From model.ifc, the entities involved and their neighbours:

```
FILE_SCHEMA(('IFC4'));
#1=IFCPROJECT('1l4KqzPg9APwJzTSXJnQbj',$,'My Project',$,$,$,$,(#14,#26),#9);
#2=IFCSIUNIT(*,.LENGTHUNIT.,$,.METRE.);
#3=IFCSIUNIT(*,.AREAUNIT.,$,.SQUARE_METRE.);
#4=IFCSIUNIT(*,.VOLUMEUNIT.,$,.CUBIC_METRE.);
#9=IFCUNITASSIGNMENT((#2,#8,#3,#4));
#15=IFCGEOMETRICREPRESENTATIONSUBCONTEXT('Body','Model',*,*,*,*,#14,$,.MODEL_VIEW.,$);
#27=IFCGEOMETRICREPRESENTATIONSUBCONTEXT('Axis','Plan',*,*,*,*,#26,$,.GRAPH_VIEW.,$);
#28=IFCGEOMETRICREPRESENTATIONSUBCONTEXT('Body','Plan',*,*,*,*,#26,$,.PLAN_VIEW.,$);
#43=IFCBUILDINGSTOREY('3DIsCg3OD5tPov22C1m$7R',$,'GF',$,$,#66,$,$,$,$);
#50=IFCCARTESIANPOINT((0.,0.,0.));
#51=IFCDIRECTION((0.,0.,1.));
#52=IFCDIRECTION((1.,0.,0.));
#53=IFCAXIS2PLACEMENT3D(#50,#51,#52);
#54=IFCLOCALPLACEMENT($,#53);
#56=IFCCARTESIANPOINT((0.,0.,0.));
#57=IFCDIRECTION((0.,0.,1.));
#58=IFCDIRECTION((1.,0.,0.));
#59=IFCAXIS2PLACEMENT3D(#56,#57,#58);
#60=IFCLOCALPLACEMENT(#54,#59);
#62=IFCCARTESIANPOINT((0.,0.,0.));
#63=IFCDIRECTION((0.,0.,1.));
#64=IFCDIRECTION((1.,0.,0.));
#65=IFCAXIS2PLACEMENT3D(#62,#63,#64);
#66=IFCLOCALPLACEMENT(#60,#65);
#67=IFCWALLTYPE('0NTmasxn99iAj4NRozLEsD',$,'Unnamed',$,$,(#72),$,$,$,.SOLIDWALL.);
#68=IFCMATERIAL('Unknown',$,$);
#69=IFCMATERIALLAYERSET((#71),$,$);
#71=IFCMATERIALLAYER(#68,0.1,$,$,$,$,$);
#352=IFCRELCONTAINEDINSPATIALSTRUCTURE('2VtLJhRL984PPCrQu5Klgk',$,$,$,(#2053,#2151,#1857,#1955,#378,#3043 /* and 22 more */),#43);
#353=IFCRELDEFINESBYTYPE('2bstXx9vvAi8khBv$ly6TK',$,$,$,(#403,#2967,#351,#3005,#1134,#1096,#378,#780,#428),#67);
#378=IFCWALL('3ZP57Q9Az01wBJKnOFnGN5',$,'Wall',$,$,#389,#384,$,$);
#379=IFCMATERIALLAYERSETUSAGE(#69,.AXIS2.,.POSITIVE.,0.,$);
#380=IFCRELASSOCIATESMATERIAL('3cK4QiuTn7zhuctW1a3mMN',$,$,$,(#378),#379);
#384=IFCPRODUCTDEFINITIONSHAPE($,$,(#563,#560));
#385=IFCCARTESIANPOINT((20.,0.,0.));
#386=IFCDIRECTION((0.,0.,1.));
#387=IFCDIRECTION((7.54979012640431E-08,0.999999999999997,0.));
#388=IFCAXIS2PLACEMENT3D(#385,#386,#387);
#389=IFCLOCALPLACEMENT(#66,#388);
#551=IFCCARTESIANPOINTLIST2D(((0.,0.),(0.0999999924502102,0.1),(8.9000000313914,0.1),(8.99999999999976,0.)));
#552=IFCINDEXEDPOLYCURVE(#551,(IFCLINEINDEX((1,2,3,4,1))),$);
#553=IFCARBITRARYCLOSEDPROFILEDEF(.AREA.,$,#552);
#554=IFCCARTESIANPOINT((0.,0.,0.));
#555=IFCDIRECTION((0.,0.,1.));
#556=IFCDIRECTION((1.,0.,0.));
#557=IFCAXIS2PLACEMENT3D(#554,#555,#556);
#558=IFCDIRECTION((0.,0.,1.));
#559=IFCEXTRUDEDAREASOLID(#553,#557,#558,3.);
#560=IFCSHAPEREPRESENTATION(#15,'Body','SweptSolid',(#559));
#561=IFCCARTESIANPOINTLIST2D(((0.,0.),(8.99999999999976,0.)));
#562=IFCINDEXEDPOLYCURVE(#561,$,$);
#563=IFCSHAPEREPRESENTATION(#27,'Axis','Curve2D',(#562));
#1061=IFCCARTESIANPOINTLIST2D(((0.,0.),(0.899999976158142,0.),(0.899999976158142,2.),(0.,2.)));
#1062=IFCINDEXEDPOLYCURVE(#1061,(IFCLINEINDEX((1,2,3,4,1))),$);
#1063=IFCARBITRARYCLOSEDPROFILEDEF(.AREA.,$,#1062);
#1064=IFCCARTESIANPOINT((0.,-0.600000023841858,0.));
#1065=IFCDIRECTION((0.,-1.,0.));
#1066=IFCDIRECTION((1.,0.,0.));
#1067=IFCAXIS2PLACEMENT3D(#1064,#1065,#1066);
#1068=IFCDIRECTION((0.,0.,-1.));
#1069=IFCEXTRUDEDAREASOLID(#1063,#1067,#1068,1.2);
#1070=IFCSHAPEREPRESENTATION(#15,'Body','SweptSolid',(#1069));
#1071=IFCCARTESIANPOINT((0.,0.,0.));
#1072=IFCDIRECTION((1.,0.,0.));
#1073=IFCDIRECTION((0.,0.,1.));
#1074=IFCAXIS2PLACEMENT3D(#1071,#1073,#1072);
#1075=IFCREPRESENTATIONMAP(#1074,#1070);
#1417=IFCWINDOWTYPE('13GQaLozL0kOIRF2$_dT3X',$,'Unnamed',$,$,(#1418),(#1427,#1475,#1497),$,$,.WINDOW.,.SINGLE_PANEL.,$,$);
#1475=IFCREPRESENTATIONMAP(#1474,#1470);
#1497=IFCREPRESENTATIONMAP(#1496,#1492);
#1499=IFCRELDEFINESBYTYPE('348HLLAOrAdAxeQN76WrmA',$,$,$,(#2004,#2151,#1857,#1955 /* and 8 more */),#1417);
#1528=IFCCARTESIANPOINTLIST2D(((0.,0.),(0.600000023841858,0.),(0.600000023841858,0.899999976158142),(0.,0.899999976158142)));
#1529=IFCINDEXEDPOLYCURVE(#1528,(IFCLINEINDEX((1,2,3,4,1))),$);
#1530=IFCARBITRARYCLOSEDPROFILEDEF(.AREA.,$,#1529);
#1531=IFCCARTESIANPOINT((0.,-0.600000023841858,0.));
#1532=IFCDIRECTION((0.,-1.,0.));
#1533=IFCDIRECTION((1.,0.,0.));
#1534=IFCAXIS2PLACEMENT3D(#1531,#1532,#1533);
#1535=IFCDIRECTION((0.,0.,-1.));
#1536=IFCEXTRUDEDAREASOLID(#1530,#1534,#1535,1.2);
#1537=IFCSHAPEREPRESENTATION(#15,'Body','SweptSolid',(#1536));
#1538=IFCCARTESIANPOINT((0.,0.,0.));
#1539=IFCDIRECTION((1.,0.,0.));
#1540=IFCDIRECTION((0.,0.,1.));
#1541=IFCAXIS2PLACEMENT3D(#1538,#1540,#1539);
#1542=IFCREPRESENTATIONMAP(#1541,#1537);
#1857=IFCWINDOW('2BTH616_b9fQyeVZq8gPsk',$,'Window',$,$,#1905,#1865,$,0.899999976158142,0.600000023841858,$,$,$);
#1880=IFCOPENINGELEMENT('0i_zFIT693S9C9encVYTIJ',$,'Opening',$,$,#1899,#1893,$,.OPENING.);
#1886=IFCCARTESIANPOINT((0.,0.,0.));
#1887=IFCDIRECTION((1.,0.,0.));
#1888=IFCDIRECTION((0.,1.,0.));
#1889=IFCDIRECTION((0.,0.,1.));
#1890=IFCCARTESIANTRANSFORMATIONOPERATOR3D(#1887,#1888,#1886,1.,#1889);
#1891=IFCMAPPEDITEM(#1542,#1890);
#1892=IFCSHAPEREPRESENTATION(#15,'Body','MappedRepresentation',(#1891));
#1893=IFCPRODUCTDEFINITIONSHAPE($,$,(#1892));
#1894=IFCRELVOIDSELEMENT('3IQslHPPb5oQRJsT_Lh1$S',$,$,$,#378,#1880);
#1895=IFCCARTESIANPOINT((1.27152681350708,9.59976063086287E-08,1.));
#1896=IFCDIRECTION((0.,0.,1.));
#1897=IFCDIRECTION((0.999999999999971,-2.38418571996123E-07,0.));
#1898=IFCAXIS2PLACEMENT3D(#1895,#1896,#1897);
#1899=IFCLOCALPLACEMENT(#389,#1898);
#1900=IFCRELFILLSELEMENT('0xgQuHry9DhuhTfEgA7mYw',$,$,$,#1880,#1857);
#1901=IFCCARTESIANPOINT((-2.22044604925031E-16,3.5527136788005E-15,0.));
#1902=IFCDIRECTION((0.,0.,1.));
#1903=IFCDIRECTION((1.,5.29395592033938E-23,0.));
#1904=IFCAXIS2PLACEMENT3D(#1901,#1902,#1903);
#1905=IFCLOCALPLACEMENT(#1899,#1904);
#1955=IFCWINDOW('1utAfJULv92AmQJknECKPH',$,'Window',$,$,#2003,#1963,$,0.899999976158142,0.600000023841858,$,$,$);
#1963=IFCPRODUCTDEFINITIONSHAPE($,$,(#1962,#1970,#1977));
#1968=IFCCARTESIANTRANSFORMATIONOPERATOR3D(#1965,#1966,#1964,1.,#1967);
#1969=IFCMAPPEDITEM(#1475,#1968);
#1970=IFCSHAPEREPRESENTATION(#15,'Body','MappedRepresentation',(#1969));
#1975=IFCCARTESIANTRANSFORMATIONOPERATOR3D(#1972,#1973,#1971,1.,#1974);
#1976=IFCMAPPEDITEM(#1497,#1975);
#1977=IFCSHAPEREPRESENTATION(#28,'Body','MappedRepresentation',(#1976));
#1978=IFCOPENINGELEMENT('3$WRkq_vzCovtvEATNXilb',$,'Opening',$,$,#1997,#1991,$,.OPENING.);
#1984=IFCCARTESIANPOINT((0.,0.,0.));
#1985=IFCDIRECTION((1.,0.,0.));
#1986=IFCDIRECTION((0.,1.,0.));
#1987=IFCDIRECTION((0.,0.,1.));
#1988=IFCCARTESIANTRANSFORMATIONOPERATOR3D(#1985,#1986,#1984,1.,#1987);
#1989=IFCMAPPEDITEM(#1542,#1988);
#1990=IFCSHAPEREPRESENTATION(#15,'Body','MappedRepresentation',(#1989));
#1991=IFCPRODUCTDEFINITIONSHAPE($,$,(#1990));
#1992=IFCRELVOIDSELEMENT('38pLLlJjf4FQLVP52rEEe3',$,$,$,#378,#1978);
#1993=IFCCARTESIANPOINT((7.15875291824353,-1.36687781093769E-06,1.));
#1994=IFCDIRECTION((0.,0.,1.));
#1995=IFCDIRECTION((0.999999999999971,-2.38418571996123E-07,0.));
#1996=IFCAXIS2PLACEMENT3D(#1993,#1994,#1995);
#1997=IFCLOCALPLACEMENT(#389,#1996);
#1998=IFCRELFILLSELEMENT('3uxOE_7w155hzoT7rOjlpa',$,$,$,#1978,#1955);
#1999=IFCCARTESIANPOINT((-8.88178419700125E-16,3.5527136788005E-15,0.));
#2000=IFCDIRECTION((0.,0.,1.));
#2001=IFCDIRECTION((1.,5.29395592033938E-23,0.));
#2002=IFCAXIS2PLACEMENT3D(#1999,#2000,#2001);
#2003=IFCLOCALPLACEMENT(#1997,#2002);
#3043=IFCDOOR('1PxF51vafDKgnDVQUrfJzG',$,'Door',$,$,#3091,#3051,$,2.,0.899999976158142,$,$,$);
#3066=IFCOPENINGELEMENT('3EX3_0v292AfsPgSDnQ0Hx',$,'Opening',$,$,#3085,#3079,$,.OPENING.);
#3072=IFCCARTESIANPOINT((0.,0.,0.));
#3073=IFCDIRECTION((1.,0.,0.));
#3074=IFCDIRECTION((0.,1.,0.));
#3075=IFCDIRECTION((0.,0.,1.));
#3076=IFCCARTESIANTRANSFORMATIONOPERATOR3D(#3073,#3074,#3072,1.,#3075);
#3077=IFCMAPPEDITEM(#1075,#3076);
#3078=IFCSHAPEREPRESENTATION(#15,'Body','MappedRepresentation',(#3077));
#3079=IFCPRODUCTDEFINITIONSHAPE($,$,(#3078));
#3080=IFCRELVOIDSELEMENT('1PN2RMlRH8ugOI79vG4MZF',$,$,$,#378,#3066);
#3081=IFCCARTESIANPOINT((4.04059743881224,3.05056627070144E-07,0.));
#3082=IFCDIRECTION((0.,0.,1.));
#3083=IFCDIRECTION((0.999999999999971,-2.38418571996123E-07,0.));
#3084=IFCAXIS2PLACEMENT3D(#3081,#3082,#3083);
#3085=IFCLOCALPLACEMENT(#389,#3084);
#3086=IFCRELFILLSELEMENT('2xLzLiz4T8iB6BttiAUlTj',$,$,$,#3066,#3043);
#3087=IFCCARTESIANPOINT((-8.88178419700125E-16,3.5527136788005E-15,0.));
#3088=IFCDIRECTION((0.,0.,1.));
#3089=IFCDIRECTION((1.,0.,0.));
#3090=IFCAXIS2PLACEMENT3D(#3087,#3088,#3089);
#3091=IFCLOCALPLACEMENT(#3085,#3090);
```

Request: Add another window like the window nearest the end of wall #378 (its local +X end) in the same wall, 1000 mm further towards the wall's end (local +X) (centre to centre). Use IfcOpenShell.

```python
import ifcopenshell
import ifcopenshell.api.feature
import ifcopenshell.api.geometry
import ifcopenshell.api.root
import ifcopenshell.geom
import ifcopenshell.util.element
import ifcopenshell.util.placement
import ifcopenshell.util.shape

model = ifcopenshell.open("model.ifc")
settings = ifcopenshell.geom.settings()


def volume(element):
    """Net volume in cubic metres, openings subtracted."""
    shape = ifcopenshell.geom.create_shape(settings, element)
    return ifcopenshell.util.shape.get_volume(shape.geometry)


window = model.by_id(1955)
opening = window.FillsVoids[0].RelatingOpeningElement
wall = opening.VoidsElements[0].RelatingBuildingElement
before = volume(wall)
shift = ifcopenshell.util.placement.get_local_placement(wall.ObjectPlacement)[:3, 0] * 1.0

# copy_class copies the void relationship, type, container and properties, but no geometry.
new_opening = ifcopenshell.api.root.copy_class(model, product=opening)
new_opening.Representation = ifcopenshell.util.element.copy_deep(
    model, opening.Representation, exclude=["IfcGeometricRepresentationContext", "IfcRepresentationMap"]
)
new_window = ifcopenshell.api.root.copy_class(model, product=window)
new_window.Representation = ifcopenshell.util.element.copy_deep(
    model, window.Representation, exclude=["IfcGeometricRepresentationContext", "IfcRepresentationMap"]
)
ifcopenshell.api.feature.add_filling(model, opening=new_opening, element=new_window)

for old, new in ((opening, new_opening), (window, new_window)):
    matrix = ifcopenshell.util.placement.get_local_placement(old.ObjectPlacement)
    matrix[:3, 3] += shift
    ifcopenshell.api.geometry.edit_object_placement(model, product=new, matrix=matrix, is_si=False)

after = volume(wall)

print(f"wall volume {before:.3f} -> {after:.3f} m3")

model.write("model-out.ifc")
```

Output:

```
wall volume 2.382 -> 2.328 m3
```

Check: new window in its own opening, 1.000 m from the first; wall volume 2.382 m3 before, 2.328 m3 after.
